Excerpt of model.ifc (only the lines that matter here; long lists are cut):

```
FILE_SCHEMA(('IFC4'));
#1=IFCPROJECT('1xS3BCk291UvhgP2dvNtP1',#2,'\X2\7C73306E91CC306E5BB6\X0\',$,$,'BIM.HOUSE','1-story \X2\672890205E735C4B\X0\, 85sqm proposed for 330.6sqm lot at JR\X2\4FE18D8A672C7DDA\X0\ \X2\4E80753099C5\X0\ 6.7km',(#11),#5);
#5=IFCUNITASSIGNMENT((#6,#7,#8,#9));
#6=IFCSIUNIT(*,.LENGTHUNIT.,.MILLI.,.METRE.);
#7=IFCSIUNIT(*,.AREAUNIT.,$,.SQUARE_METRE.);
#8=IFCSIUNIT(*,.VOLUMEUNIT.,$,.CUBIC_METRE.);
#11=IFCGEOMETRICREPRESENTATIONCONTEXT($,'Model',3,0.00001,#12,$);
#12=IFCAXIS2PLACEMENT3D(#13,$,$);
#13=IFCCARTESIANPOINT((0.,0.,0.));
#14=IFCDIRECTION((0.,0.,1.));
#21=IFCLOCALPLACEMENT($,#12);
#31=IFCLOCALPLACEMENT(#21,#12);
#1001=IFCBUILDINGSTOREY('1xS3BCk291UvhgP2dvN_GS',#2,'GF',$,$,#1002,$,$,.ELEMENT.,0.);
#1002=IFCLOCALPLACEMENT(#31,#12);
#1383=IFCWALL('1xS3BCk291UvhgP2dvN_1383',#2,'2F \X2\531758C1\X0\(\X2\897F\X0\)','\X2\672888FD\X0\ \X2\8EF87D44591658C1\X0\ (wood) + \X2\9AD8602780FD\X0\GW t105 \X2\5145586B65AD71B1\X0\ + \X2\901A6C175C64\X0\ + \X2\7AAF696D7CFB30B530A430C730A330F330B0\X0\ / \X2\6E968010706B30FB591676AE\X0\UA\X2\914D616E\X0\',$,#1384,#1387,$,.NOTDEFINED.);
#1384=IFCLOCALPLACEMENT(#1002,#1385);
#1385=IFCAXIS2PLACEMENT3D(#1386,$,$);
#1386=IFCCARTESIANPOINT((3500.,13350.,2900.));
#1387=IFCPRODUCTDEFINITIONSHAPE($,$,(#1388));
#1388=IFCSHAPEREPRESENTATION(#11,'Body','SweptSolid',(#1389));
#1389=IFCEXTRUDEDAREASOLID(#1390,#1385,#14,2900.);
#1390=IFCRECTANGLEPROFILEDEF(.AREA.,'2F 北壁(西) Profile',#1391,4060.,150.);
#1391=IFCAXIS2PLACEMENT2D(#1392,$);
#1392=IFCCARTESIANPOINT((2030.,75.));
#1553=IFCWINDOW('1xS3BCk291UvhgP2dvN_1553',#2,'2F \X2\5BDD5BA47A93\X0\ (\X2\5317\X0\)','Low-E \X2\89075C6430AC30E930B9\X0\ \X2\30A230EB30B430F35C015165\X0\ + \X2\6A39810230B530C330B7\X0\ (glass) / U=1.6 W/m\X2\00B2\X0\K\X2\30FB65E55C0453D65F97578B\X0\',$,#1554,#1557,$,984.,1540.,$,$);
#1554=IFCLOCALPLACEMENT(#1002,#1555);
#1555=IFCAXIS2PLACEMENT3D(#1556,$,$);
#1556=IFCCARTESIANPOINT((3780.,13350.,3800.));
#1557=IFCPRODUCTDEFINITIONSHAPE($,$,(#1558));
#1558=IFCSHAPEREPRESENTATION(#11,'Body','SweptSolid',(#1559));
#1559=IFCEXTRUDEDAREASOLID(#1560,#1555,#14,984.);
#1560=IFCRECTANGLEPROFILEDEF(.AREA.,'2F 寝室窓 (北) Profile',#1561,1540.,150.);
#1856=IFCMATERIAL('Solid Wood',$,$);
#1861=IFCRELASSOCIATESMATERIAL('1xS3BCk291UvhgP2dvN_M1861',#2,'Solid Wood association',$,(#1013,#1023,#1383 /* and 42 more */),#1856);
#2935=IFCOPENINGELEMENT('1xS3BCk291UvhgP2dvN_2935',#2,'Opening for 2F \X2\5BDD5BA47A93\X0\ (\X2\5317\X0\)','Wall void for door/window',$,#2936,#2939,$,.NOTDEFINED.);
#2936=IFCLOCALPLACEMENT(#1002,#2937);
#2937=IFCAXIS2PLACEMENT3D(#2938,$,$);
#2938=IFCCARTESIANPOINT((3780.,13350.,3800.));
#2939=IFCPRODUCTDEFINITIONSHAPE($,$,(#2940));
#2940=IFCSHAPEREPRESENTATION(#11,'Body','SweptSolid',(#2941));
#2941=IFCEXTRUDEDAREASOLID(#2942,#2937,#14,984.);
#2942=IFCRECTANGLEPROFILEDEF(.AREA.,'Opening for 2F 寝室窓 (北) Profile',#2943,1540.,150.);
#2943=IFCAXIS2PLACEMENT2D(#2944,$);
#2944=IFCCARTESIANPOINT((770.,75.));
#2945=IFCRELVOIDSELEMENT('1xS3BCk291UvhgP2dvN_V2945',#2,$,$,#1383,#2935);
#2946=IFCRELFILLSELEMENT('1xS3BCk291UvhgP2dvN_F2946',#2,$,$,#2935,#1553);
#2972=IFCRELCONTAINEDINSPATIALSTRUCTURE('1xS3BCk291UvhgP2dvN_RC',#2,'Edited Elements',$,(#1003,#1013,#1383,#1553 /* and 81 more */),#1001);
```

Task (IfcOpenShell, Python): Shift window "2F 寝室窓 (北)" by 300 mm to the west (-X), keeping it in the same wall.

```python
import ifcopenshell
import ifcopenshell.api.geometry
import ifcopenshell.util.placement

model = ifcopenshell.open("model.ifc")

window = model.by_guid("1xS3BCk291UvhgP2dvN_1553")
opening = window.FillsVoids[0].RelatingOpeningElement
wall = opening.VoidsElements[0].RelatingBuildingElement

wall_matrix = ifcopenshell.util.placement.get_local_placement(wall.ObjectPlacement)
shift = wall_matrix[:3, 0] * -300.0
before = ifcopenshell.util.placement.get_local_placement(window.ObjectPlacement)[:3, 3].copy()

# The window is not placed relative to its opening, so move both.
for product in (opening, window):
    matrix = ifcopenshell.util.placement.get_local_placement(product.ObjectPlacement)
    matrix[:3, 3] += shift
    ifcopenshell.api.geometry.edit_object_placement(model, product=product, matrix=matrix, is_si=False)

after = ifcopenshell.util.placement.get_local_placement(window.ObjectPlacement)[:3, 3]
print("window moved by", (after - before).round(3) + 0.0)

model.write("model_edited.ifc")
```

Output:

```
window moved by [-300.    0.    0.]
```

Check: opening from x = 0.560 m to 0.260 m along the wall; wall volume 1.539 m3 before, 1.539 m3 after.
